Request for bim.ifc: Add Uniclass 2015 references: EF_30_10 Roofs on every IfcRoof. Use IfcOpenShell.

First a look at what the model holds.

```python
import ifcopenshell

model = ifcopenshell.open("bim.ifc")
print(model.schema)
print("classifications:", [c.Name for c in model.by_type("IfcClassification")])
for ifc_class in ("IfcDoor", "IfcRoof", "IfcStair", "IfcWall", "IfcWindow"):
    print(ifc_class, len(model.by_type(ifc_class)))
```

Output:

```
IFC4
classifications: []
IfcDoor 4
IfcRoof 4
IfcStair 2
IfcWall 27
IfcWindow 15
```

```python
import ifcopenshell
import ifcopenshell.api.classification

model = ifcopenshell.open("bim.ifc")

system = ifcopenshell.api.classification.add_classification(model, classification="Uniclass 2015")

codes = {
    "IfcRoof": ("EF_30_10", "Roofs"),
}
for ifc_class, (code, name) in codes.items():
    products = model.by_type(ifc_class)
    ifcopenshell.api.classification.add_reference(
        model, products=products, classification=system, identification=code, name=name
    )
    print(code, len(products))

model.write("bim_rev.ifc")
```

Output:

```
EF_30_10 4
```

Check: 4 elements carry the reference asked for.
